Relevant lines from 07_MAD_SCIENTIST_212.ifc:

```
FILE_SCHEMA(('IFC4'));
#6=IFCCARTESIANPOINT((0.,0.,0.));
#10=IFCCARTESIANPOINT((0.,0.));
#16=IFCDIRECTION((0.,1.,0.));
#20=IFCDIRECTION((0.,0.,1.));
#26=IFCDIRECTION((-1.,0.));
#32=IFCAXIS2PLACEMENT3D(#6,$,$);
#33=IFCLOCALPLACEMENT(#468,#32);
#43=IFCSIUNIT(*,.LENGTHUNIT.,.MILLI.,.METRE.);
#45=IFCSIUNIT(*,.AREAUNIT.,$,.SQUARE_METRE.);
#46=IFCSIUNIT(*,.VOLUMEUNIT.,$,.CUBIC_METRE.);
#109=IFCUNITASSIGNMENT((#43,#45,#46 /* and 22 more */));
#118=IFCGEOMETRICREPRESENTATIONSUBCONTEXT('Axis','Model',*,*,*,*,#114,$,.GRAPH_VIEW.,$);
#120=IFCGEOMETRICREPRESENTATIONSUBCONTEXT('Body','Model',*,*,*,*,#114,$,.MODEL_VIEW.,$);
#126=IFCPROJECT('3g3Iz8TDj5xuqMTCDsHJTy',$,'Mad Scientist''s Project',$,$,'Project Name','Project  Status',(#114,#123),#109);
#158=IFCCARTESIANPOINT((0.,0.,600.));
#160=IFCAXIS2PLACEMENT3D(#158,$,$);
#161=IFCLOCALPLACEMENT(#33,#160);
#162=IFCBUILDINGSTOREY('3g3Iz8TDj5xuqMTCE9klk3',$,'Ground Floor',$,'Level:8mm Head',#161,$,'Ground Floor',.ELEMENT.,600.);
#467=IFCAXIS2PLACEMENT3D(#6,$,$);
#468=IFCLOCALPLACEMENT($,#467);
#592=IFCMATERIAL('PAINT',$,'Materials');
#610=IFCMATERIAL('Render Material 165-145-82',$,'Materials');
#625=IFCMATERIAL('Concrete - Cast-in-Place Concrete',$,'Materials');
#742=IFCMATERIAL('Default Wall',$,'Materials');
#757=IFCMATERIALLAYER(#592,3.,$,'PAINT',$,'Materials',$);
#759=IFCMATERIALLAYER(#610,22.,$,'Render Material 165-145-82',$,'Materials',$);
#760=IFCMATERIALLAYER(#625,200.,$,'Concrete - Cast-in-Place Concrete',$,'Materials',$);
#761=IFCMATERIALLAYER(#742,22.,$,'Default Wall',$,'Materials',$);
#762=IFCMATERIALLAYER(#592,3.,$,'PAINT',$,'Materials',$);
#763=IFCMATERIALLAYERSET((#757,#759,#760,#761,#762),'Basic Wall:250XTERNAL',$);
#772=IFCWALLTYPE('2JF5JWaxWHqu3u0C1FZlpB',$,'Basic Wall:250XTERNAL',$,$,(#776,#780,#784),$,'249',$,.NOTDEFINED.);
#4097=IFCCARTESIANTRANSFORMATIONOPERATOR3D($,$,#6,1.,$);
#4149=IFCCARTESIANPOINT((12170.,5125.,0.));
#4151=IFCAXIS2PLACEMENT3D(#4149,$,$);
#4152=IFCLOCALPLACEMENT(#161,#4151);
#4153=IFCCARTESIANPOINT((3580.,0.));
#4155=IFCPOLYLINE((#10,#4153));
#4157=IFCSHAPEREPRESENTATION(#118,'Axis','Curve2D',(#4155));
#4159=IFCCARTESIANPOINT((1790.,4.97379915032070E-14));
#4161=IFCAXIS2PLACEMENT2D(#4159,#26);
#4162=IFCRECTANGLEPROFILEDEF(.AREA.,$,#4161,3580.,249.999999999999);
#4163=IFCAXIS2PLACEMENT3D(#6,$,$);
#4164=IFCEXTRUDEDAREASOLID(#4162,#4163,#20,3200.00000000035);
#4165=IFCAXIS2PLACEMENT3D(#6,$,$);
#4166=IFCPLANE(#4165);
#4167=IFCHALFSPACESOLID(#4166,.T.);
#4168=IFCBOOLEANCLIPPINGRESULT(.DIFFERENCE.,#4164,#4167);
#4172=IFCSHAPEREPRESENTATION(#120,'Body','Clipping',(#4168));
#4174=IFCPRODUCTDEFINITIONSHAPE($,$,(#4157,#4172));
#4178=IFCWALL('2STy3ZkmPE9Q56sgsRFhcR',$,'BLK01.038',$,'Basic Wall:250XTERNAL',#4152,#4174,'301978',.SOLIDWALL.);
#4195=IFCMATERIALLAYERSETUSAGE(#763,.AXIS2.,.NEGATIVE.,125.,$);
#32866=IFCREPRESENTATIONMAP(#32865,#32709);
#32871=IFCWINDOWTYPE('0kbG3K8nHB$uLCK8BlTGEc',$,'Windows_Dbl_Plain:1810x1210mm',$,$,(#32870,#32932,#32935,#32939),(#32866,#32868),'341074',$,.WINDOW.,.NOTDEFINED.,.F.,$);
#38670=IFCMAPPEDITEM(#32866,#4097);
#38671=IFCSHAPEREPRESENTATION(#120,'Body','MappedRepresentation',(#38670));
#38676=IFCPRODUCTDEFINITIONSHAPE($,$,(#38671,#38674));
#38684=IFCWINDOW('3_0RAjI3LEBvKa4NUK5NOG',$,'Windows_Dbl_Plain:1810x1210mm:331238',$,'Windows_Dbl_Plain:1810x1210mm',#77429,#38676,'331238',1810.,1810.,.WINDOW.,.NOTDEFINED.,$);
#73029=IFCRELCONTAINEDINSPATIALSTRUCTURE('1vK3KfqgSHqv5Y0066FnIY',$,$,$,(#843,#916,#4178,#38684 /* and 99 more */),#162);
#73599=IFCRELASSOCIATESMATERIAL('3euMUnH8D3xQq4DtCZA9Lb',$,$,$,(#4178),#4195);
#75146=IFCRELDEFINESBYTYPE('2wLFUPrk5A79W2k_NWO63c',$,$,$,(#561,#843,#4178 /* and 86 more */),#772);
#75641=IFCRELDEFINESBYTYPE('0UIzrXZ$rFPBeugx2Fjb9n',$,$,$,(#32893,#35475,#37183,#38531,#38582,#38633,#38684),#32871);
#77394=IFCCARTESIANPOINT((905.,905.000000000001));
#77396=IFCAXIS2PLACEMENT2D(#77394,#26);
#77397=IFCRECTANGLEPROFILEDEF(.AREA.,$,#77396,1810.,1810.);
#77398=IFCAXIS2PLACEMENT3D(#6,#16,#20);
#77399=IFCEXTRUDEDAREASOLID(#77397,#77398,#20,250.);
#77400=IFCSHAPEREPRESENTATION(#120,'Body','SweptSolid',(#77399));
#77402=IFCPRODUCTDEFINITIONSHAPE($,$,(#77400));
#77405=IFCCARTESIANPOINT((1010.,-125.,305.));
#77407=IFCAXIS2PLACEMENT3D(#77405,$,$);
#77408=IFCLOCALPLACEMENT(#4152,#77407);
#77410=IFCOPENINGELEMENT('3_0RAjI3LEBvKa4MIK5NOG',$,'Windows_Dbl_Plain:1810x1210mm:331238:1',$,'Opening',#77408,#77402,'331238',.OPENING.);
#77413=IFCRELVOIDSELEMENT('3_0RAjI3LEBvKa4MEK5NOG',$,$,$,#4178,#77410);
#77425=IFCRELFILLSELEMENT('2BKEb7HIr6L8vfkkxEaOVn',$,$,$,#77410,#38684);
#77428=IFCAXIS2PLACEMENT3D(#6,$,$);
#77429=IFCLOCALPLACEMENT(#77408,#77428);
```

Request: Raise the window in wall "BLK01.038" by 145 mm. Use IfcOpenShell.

```python
import numpy as np
import ifcopenshell
import ifcopenshell.api.geometry
import ifcopenshell.util.placement
import ifcopenshell.util.unit

model = ifcopenshell.open("07_MAD_SCIENTIST_212.ifc")
unit_scale = ifcopenshell.util.unit.calculate_unit_scale(model)

window = model.by_guid("3_0RAjI3LEBvKa4NUK5NOG")
opening = window.FillsVoids[0].RelatingOpeningElement
dz = 145.0

shift = np.array([0.0, 0.0, dz])
# The window is placed relative to its opening, so it follows when the opening moves.
matrix = ifcopenshell.util.placement.get_local_placement(opening.ObjectPlacement)
matrix[:3, 3] += shift
ifcopenshell.api.geometry.edit_object_placement(
    model, product=opening, matrix=matrix, is_si=False, should_transform_children=True
)

print(f"moved by {dz * unit_scale:+.3f} m")

model.write("07_MAD_SCIENTIST_212_updated.ifc")
```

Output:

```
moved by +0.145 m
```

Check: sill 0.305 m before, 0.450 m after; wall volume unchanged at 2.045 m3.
